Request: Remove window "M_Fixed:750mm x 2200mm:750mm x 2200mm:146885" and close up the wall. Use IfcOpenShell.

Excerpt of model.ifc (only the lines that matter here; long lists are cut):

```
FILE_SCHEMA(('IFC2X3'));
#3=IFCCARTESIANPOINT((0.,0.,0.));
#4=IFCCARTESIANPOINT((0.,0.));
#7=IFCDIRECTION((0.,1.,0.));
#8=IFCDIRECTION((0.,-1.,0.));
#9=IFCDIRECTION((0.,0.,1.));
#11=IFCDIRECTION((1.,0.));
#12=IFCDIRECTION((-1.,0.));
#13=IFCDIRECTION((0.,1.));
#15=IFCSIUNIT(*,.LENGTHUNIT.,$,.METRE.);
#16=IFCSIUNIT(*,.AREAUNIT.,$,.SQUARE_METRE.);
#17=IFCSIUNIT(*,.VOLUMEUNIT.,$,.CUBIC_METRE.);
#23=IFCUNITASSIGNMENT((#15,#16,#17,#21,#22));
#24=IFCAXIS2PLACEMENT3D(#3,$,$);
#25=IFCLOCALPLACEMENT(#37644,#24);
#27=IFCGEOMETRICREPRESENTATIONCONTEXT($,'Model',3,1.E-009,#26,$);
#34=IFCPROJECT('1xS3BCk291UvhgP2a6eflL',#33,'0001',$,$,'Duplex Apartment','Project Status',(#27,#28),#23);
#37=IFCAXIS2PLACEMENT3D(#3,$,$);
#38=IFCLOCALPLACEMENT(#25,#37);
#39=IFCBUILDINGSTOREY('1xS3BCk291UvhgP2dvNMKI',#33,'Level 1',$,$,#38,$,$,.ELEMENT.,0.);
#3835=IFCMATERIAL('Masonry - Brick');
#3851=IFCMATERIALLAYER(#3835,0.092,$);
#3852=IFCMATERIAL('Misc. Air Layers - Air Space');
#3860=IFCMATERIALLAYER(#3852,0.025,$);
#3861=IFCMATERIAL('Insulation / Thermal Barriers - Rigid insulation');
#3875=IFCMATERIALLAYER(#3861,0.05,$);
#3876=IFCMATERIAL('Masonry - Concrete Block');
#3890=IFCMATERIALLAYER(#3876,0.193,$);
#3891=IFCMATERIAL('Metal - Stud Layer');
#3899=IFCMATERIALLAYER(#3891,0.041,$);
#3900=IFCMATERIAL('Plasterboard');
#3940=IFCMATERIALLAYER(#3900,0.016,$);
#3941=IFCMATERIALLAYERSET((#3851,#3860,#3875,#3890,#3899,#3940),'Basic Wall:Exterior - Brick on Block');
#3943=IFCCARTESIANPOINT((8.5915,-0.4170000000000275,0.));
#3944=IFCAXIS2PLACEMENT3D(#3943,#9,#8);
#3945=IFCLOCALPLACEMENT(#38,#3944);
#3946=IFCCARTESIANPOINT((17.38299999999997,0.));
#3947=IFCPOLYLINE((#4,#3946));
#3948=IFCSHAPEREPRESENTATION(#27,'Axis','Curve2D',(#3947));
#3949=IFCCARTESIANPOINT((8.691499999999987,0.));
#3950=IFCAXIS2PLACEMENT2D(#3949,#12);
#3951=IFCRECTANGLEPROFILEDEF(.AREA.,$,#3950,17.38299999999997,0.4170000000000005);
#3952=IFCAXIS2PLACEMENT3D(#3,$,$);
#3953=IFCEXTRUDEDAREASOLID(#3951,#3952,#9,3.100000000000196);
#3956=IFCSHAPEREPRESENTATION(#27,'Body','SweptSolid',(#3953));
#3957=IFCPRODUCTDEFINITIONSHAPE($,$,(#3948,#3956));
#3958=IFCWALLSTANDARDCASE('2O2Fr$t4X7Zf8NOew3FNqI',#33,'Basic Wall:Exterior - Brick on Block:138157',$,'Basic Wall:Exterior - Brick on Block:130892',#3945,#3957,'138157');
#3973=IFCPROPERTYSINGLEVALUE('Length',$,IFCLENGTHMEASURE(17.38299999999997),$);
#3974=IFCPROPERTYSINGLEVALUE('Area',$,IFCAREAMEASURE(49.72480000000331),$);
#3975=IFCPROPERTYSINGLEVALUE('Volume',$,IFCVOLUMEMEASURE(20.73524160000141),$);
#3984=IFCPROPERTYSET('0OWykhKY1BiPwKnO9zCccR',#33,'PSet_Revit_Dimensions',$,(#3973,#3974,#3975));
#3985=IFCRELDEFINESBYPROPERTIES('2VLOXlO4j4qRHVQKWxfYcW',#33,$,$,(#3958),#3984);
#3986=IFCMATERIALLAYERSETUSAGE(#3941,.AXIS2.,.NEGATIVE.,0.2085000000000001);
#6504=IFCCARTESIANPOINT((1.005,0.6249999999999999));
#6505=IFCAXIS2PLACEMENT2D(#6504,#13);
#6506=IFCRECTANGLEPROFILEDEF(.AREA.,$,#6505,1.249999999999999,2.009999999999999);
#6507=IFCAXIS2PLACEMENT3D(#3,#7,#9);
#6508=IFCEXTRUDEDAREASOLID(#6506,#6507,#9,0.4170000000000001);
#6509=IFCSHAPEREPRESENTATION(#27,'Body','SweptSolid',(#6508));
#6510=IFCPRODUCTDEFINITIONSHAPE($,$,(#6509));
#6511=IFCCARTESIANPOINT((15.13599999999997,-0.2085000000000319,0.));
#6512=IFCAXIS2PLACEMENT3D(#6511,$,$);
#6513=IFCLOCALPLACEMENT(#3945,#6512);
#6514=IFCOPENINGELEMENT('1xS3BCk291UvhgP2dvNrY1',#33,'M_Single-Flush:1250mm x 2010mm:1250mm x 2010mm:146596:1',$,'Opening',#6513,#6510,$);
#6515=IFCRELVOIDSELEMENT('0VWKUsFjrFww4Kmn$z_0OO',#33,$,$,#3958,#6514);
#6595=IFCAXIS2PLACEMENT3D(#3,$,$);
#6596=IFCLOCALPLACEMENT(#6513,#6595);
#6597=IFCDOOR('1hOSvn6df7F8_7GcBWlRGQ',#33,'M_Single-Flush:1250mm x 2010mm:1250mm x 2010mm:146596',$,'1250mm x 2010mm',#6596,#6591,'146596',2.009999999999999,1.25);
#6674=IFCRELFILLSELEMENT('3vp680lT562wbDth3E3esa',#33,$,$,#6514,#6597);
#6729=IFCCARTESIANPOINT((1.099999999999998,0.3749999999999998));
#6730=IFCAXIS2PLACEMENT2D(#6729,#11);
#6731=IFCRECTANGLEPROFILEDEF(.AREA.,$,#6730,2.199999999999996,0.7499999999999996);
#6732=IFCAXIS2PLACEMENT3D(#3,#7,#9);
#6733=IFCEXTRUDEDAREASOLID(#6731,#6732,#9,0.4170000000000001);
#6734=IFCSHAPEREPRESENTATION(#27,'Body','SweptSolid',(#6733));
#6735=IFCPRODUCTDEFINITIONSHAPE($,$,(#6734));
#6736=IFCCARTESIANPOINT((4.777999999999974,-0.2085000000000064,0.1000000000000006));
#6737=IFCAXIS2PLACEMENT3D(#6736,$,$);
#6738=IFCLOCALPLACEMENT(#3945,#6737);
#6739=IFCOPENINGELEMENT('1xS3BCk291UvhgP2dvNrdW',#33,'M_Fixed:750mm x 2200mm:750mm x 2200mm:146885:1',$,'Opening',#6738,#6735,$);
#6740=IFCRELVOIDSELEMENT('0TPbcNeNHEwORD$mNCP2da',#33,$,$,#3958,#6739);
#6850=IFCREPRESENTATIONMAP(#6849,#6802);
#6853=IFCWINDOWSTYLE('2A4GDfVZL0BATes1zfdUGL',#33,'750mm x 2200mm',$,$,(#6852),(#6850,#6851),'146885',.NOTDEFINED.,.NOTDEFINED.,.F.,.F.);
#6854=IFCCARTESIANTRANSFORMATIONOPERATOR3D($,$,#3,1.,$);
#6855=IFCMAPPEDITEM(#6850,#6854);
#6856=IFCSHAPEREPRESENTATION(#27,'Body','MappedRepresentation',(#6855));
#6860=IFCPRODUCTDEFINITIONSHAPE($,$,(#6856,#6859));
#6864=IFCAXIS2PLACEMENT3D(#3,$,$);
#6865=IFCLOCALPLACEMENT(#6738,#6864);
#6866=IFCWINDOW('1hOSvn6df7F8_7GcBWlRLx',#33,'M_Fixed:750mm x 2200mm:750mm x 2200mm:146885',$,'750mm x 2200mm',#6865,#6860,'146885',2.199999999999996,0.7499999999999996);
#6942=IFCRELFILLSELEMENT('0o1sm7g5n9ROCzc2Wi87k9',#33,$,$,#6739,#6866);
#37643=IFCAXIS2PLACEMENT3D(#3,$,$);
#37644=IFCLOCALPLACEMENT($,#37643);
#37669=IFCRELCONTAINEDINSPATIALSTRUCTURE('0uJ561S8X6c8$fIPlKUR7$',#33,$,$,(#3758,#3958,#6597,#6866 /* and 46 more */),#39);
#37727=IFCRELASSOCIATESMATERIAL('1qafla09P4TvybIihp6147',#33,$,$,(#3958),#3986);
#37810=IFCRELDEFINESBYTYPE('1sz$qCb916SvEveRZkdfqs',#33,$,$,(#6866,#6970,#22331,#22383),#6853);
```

```python
import ifcopenshell
import ifcopenshell.api.feature
import ifcopenshell.api.pset
import ifcopenshell.api.root
import ifcopenshell.geom
import ifcopenshell.util.element
import ifcopenshell.util.shape
import ifcopenshell.util.unit

model = ifcopenshell.open("model.ifc")
area_scale = ifcopenshell.util.unit.calculate_unit_scale(model, "AREAUNIT")
volume_scale = ifcopenshell.util.unit.calculate_unit_scale(model, "VOLUMEUNIT")
settings = ifcopenshell.geom.settings()


def volume(element):
    """Net volume in cubic metres, openings subtracted."""
    shape = ifcopenshell.geom.create_shape(settings, element)
    return ifcopenshell.util.shape.get_volume(shape.geometry)


window = model.by_id(6866)
opening = window.FillsVoids[0].RelatingOpeningElement
wall = opening.VoidsElements[0].RelatingBuildingElement
before = volume(wall)

ifcopenshell.api.root.remove_product(model, product=window)
ifcopenshell.api.feature.remove_feature(model, feature=opening)

after = volume(wall)
thickness = 0.417  # wall thickness in metres

# Update the wall's stored quantities.
pset = model.by_id(ifcopenshell.util.element.get_pset(wall, "PSet_Revit_Dimensions", should_inherit=False)["id"])
ifcopenshell.api.pset.edit_pset(model, pset=pset, properties={
    "Area": model.create_entity("IfcAreaMeasure", after / thickness / area_scale),
    "Volume": model.create_entity("IfcVolumeMeasure", after / volume_scale),
})

print(f"wall volume {before:.3f} -> {after:.3f} m3")

model.write("model_rev.ifc")
```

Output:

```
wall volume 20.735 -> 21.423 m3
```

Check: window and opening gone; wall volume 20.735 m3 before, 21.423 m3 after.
